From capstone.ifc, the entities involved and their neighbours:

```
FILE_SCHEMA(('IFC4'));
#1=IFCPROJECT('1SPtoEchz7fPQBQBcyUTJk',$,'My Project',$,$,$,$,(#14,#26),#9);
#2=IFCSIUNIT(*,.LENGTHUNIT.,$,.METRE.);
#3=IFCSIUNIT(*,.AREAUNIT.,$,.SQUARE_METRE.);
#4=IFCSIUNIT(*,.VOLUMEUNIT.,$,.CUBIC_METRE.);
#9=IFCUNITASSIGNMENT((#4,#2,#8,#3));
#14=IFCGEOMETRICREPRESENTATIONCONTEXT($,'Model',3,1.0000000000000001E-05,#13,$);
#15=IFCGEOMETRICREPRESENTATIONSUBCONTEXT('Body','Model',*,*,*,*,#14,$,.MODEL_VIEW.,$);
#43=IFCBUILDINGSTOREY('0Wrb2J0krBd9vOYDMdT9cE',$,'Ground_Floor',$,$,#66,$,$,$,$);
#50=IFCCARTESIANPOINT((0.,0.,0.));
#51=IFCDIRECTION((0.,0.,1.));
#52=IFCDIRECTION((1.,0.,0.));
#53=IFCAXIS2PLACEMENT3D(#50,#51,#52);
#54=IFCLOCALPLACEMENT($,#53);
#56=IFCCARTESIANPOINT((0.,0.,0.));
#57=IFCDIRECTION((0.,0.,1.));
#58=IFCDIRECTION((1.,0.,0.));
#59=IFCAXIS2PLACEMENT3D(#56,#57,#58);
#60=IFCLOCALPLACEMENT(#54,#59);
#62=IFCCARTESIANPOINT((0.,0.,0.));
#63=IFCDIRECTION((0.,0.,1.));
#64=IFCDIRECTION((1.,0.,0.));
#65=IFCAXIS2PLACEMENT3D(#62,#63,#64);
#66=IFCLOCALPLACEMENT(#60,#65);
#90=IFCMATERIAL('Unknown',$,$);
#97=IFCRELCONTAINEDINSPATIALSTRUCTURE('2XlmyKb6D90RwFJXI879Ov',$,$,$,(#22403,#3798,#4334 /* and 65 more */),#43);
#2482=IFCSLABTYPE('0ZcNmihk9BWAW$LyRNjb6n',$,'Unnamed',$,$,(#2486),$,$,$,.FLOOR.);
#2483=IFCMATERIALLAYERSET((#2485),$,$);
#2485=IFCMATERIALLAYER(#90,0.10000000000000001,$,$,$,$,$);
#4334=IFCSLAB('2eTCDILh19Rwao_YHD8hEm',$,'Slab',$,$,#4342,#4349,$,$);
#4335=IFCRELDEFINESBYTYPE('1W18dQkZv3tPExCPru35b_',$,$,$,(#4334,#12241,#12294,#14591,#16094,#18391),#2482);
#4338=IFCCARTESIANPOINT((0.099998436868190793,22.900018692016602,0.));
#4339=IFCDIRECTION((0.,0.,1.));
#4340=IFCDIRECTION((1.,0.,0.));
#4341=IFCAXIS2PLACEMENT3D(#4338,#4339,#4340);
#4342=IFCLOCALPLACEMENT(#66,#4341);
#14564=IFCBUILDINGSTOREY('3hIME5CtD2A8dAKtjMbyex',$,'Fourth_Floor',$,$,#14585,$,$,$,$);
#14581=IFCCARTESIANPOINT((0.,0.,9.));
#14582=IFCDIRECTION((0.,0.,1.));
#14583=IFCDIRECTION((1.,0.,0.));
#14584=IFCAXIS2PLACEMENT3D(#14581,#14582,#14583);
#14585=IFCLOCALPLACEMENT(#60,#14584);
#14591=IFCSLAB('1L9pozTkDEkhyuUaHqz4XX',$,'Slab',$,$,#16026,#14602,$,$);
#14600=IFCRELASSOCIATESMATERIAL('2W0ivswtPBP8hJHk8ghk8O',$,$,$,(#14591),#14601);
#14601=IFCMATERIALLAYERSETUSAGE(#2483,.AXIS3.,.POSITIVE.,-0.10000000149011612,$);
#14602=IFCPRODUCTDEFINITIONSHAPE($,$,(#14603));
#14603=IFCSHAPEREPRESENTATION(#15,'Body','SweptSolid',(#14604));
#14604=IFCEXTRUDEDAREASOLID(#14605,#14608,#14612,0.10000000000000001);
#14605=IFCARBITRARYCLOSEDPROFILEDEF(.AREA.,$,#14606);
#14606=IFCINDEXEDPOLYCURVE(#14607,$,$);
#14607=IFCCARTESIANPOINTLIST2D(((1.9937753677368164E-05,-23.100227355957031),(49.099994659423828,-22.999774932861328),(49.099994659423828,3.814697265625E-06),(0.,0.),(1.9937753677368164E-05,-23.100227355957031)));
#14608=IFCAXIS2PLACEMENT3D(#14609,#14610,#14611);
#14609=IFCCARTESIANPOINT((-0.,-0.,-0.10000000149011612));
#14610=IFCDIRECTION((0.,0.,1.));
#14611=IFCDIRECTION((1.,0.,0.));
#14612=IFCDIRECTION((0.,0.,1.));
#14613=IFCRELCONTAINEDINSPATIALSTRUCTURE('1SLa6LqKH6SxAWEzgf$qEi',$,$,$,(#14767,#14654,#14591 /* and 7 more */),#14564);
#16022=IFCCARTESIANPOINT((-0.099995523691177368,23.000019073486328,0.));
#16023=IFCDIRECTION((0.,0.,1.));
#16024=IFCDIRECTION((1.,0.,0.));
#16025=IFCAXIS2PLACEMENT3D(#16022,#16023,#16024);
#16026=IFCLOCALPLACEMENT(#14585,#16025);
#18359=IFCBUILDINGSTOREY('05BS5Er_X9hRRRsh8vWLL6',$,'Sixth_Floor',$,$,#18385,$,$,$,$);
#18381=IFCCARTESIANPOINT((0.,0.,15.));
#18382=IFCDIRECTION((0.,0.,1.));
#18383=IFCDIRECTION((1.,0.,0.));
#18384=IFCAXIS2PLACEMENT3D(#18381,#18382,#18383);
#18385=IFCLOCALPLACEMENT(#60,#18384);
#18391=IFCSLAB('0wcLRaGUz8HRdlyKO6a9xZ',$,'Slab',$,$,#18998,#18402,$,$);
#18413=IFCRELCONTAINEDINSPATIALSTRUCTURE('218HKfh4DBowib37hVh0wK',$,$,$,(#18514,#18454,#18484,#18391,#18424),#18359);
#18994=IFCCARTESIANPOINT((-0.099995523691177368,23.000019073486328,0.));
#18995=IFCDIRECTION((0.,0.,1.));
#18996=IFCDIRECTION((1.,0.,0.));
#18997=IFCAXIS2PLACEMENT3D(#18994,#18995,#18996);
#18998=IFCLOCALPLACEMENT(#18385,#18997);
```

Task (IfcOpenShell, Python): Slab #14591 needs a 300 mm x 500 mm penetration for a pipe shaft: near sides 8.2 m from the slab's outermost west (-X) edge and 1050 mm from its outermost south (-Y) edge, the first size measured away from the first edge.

```python
import numpy as np
import ifcopenshell
import ifcopenshell.api.feature
import ifcopenshell.api.geometry
import ifcopenshell.api.root
import ifcopenshell.geom
import ifcopenshell.util.placement
import ifcopenshell.util.representation
import ifcopenshell.util.shape
import ifcopenshell.util.unit

model = ifcopenshell.open("capstone.ifc")
unit_scale = ifcopenshell.util.unit.calculate_unit_scale(model)
settings = ifcopenshell.geom.settings()


def volume(element):
    """Net volume in cubic metres, openings subtracted."""
    shape = ifcopenshell.geom.create_shape(settings, element)
    return ifcopenshell.util.shape.get_volume(shape.geometry)


slab = model.by_guid("1L9pozTkDEkhyuUaHqz4XX")
before = volume(slab)

# Extent in the slab's own axes, in metres. The edges named are its -X and -Y sides.
slab_shape = ifcopenshell.geom.create_shape(settings, slab)
vertices = ifcopenshell.util.shape.get_vertices(slab_shape.geometry)
x_min, y_min, bottom = vertices.min(axis=0)
top = vertices[:, 2].max()

opening = ifcopenshell.api.root.create_entity(model, ifc_class="IfcOpeningElement", name="Pipe shaft opening", predefined_type="OPENING")
context = ifcopenshell.util.representation.get_context(model, "Model", "Body", "MODEL_VIEW")
width, depth = 0.3, 0.5
outline = [(0.0, 0.0), (width, 0.0), (width, depth), (0.0, depth), (0.0, 0.0)]
# Overshoot both faces by 50 mm so the cut is clean.
shape = ifcopenshell.api.geometry.add_slab_representation(
    model, context=context, depth=top - bottom + 0.1, polyline=outline
)
ifcopenshell.api.geometry.assign_representation(model, product=opening, representation=shape)

matrix = ifcopenshell.util.placement.get_local_placement(slab.ObjectPlacement)
matrix[:, 3] = matrix @ np.append(np.array([x_min + 8.2, y_min + 1.05, bottom - 0.05]) / unit_scale, 1.0)
ifcopenshell.api.geometry.edit_object_placement(model, product=opening, matrix=matrix, is_si=False)
ifcopenshell.api.feature.add_feature(model, feature=opening, element=slab)

after = volume(slab)

print(f"slab volume {before:.3f} -> {after:.3f} m3")

model.write("capstone_rev.ifc")
```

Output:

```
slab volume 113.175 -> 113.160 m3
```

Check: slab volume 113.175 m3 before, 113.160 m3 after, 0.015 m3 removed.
